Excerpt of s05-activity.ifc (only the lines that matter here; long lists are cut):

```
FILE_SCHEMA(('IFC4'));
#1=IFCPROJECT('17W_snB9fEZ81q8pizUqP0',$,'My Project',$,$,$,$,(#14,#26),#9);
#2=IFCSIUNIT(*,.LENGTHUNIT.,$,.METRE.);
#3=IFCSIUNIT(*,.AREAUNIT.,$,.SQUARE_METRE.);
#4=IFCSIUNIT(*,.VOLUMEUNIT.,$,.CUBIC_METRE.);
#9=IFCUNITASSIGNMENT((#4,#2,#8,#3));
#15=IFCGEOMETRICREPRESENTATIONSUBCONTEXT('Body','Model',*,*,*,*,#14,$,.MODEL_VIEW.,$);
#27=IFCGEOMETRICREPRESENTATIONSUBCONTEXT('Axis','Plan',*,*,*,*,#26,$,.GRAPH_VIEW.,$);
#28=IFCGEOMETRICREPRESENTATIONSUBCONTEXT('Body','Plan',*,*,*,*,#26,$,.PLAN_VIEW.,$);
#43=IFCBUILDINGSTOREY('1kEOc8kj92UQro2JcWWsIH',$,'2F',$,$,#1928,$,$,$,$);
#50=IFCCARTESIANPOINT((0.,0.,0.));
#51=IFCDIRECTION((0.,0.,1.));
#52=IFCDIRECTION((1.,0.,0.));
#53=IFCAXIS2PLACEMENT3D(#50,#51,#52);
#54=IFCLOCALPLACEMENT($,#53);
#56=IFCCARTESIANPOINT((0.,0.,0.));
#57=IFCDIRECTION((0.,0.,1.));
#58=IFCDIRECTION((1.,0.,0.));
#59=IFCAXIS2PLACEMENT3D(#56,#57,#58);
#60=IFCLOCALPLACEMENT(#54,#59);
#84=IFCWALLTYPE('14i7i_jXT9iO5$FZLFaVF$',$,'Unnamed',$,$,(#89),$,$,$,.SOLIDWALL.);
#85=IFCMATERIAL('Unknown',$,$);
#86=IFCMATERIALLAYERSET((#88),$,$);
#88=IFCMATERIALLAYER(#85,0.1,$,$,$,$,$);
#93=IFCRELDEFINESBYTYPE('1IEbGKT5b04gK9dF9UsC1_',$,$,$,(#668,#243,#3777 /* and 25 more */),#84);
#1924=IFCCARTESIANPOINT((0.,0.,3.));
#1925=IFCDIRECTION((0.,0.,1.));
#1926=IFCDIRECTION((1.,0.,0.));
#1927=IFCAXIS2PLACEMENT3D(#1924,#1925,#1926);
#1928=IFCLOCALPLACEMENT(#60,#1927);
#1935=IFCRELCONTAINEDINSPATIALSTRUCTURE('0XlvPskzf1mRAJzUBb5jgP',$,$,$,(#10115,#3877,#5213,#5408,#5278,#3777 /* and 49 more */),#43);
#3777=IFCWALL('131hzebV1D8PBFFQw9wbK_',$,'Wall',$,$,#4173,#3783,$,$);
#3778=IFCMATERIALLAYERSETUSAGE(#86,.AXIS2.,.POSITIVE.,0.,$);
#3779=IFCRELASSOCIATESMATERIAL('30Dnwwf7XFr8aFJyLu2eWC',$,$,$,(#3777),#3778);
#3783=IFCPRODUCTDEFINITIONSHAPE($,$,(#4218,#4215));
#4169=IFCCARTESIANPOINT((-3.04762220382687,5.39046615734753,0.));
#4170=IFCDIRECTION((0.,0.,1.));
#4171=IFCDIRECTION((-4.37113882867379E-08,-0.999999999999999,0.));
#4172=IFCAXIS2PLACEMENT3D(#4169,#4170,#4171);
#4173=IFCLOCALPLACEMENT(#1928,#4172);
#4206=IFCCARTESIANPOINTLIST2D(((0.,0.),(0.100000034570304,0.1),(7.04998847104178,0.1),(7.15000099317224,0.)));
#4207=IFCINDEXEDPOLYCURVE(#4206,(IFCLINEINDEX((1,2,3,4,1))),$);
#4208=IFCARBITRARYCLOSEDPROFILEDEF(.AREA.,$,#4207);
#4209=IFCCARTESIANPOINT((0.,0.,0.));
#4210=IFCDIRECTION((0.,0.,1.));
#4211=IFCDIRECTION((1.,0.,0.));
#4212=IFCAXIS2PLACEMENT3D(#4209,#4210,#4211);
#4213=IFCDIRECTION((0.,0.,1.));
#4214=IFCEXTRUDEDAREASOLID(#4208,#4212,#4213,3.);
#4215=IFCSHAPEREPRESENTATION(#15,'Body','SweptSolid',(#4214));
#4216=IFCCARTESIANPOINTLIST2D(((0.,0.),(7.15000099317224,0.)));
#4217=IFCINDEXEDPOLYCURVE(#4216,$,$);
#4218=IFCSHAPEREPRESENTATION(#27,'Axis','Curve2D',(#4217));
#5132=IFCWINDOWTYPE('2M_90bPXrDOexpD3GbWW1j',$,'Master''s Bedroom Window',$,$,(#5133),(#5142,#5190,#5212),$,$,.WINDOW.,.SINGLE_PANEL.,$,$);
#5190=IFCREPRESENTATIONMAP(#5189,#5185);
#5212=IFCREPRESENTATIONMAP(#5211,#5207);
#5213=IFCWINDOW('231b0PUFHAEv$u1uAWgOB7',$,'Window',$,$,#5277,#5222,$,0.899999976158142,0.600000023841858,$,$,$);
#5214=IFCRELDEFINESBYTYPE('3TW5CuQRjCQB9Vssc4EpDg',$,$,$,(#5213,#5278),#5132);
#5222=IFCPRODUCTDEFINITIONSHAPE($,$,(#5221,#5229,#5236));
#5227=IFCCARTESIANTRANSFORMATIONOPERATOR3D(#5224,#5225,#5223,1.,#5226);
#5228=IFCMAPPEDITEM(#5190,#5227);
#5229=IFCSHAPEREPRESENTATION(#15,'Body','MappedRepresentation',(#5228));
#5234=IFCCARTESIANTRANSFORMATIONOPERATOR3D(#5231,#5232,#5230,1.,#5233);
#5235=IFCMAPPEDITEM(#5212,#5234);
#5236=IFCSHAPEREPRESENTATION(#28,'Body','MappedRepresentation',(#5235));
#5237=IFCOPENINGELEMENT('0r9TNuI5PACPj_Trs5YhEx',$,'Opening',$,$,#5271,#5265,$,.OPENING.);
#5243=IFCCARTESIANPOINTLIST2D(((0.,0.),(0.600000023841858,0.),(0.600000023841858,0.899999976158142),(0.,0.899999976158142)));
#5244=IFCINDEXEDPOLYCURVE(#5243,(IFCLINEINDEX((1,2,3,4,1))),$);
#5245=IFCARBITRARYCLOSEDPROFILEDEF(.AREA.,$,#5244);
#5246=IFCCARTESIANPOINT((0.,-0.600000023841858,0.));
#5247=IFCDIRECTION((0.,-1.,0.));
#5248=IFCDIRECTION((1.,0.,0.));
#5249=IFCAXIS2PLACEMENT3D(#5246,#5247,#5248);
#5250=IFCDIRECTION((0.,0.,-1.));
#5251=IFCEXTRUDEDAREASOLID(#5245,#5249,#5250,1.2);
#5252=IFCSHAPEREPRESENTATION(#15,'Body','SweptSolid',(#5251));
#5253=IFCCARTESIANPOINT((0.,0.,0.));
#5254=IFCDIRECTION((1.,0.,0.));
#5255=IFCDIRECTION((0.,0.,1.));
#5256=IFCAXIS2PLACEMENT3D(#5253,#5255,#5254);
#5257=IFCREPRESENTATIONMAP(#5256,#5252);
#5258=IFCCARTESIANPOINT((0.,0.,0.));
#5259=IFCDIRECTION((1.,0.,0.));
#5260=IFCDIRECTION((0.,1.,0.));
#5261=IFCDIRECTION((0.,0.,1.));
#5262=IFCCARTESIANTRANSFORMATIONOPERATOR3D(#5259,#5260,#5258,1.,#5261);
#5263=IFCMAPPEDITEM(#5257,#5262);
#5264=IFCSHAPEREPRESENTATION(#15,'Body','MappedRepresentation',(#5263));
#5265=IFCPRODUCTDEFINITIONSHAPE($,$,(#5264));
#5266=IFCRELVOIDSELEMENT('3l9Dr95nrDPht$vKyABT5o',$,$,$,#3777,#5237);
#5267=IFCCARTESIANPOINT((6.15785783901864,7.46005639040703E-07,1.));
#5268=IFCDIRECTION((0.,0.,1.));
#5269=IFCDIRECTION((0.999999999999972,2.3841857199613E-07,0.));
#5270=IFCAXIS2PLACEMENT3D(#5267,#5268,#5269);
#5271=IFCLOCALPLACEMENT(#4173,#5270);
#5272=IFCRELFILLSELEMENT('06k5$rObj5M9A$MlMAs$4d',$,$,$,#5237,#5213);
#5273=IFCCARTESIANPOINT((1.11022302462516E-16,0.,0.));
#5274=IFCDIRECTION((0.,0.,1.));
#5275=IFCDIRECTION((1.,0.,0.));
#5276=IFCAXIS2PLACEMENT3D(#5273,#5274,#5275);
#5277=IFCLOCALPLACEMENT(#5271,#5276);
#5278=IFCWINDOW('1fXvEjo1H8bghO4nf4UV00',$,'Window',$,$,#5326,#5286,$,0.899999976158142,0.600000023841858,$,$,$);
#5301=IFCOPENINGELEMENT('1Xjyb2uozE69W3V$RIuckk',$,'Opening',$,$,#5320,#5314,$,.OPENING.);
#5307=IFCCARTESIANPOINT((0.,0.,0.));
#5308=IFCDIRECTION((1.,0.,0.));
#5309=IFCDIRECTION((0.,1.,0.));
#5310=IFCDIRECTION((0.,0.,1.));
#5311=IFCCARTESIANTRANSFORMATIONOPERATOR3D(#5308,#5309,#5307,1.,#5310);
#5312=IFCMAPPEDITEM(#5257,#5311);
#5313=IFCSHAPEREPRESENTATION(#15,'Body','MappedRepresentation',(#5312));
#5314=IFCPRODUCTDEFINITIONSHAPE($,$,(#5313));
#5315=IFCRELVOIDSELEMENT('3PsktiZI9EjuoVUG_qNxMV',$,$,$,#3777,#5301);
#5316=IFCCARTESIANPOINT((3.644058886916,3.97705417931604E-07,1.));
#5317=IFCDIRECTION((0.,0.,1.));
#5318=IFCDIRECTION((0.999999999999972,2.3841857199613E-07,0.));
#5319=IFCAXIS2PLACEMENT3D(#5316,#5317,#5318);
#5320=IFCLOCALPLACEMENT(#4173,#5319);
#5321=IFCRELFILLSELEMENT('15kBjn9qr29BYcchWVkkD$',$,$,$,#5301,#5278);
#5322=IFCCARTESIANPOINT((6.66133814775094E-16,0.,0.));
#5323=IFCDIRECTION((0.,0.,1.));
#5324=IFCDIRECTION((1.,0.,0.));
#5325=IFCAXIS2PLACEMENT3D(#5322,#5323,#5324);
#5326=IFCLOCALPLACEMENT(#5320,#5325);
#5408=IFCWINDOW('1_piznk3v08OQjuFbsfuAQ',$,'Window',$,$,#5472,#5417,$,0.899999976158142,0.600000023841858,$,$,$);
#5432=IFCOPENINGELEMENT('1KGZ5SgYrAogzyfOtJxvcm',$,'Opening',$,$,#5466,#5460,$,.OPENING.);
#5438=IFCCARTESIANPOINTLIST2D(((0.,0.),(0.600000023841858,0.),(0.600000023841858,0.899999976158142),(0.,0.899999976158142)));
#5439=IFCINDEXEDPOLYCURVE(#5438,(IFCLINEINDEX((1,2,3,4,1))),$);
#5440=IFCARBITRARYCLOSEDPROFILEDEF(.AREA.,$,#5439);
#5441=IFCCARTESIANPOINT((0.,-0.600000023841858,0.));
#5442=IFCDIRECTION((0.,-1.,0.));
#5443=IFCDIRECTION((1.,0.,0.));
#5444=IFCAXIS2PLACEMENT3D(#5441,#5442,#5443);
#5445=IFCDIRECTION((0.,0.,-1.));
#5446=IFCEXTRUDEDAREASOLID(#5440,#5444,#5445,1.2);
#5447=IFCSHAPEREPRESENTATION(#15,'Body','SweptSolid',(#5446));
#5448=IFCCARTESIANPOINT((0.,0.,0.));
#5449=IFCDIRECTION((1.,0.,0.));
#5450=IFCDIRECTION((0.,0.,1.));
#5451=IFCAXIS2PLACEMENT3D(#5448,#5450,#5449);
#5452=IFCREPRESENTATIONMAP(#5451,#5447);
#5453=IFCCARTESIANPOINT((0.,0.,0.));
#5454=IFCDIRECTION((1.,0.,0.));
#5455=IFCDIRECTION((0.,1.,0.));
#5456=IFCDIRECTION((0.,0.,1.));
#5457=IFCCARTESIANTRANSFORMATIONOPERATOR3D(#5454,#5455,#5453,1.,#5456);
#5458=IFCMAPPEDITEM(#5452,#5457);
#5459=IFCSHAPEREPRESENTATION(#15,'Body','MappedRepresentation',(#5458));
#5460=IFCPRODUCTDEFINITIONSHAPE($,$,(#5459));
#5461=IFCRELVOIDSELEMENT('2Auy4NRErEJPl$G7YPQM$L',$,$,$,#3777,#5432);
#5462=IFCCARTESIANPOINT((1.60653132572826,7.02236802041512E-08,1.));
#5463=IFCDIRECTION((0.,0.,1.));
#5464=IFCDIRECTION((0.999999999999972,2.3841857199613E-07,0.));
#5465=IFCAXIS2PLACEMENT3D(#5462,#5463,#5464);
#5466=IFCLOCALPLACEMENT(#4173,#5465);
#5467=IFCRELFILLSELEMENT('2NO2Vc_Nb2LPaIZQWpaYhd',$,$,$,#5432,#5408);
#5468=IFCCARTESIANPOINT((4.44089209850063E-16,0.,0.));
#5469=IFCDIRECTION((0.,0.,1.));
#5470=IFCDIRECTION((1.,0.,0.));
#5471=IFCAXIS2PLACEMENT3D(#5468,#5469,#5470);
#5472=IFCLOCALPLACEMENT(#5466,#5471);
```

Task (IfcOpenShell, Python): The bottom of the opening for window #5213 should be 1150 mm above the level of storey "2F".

```python
import numpy as np
import ifcopenshell
import ifcopenshell.api.geometry
import ifcopenshell.geom
import ifcopenshell.util.element
import ifcopenshell.util.placement
import ifcopenshell.util.shape
import ifcopenshell.util.unit

model = ifcopenshell.open("s05-activity.ifc")
unit_scale = ifcopenshell.util.unit.calculate_unit_scale(model)

window = model.by_guid("231b0PUFHAEv$u1uAWgOB7")
opening = window.FillsVoids[0].RelatingOpeningElement
storey = ifcopenshell.util.element.get_container(window, ifc_class="IfcBuildingStorey")
level = ifcopenshell.util.placement.get_local_placement(storey.ObjectPlacement)[2, 3]

# The opening's origin need not be at the sill, so measure its lowest point.
shape = ifcopenshell.geom.create_shape(ifcopenshell.geom.settings(), opening)
bottom = ifcopenshell.util.shape.get_shape_bottom_elevation(shape, shape.geometry) / unit_scale
dz = level + 1.15 / unit_scale - bottom

shift = np.array([0.0, 0.0, dz])
# The window is placed relative to its opening, so it follows when the opening moves.
matrix = ifcopenshell.util.placement.get_local_placement(opening.ObjectPlacement)
matrix[:3, 3] += shift
ifcopenshell.api.geometry.edit_object_placement(
    model, product=opening, matrix=matrix, is_si=False, should_transform_children=True
)

print(f"moved by {dz * unit_scale:+.3f} m")

model.write("s05-activity_rev.ifc")
```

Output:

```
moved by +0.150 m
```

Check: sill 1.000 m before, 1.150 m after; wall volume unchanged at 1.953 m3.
